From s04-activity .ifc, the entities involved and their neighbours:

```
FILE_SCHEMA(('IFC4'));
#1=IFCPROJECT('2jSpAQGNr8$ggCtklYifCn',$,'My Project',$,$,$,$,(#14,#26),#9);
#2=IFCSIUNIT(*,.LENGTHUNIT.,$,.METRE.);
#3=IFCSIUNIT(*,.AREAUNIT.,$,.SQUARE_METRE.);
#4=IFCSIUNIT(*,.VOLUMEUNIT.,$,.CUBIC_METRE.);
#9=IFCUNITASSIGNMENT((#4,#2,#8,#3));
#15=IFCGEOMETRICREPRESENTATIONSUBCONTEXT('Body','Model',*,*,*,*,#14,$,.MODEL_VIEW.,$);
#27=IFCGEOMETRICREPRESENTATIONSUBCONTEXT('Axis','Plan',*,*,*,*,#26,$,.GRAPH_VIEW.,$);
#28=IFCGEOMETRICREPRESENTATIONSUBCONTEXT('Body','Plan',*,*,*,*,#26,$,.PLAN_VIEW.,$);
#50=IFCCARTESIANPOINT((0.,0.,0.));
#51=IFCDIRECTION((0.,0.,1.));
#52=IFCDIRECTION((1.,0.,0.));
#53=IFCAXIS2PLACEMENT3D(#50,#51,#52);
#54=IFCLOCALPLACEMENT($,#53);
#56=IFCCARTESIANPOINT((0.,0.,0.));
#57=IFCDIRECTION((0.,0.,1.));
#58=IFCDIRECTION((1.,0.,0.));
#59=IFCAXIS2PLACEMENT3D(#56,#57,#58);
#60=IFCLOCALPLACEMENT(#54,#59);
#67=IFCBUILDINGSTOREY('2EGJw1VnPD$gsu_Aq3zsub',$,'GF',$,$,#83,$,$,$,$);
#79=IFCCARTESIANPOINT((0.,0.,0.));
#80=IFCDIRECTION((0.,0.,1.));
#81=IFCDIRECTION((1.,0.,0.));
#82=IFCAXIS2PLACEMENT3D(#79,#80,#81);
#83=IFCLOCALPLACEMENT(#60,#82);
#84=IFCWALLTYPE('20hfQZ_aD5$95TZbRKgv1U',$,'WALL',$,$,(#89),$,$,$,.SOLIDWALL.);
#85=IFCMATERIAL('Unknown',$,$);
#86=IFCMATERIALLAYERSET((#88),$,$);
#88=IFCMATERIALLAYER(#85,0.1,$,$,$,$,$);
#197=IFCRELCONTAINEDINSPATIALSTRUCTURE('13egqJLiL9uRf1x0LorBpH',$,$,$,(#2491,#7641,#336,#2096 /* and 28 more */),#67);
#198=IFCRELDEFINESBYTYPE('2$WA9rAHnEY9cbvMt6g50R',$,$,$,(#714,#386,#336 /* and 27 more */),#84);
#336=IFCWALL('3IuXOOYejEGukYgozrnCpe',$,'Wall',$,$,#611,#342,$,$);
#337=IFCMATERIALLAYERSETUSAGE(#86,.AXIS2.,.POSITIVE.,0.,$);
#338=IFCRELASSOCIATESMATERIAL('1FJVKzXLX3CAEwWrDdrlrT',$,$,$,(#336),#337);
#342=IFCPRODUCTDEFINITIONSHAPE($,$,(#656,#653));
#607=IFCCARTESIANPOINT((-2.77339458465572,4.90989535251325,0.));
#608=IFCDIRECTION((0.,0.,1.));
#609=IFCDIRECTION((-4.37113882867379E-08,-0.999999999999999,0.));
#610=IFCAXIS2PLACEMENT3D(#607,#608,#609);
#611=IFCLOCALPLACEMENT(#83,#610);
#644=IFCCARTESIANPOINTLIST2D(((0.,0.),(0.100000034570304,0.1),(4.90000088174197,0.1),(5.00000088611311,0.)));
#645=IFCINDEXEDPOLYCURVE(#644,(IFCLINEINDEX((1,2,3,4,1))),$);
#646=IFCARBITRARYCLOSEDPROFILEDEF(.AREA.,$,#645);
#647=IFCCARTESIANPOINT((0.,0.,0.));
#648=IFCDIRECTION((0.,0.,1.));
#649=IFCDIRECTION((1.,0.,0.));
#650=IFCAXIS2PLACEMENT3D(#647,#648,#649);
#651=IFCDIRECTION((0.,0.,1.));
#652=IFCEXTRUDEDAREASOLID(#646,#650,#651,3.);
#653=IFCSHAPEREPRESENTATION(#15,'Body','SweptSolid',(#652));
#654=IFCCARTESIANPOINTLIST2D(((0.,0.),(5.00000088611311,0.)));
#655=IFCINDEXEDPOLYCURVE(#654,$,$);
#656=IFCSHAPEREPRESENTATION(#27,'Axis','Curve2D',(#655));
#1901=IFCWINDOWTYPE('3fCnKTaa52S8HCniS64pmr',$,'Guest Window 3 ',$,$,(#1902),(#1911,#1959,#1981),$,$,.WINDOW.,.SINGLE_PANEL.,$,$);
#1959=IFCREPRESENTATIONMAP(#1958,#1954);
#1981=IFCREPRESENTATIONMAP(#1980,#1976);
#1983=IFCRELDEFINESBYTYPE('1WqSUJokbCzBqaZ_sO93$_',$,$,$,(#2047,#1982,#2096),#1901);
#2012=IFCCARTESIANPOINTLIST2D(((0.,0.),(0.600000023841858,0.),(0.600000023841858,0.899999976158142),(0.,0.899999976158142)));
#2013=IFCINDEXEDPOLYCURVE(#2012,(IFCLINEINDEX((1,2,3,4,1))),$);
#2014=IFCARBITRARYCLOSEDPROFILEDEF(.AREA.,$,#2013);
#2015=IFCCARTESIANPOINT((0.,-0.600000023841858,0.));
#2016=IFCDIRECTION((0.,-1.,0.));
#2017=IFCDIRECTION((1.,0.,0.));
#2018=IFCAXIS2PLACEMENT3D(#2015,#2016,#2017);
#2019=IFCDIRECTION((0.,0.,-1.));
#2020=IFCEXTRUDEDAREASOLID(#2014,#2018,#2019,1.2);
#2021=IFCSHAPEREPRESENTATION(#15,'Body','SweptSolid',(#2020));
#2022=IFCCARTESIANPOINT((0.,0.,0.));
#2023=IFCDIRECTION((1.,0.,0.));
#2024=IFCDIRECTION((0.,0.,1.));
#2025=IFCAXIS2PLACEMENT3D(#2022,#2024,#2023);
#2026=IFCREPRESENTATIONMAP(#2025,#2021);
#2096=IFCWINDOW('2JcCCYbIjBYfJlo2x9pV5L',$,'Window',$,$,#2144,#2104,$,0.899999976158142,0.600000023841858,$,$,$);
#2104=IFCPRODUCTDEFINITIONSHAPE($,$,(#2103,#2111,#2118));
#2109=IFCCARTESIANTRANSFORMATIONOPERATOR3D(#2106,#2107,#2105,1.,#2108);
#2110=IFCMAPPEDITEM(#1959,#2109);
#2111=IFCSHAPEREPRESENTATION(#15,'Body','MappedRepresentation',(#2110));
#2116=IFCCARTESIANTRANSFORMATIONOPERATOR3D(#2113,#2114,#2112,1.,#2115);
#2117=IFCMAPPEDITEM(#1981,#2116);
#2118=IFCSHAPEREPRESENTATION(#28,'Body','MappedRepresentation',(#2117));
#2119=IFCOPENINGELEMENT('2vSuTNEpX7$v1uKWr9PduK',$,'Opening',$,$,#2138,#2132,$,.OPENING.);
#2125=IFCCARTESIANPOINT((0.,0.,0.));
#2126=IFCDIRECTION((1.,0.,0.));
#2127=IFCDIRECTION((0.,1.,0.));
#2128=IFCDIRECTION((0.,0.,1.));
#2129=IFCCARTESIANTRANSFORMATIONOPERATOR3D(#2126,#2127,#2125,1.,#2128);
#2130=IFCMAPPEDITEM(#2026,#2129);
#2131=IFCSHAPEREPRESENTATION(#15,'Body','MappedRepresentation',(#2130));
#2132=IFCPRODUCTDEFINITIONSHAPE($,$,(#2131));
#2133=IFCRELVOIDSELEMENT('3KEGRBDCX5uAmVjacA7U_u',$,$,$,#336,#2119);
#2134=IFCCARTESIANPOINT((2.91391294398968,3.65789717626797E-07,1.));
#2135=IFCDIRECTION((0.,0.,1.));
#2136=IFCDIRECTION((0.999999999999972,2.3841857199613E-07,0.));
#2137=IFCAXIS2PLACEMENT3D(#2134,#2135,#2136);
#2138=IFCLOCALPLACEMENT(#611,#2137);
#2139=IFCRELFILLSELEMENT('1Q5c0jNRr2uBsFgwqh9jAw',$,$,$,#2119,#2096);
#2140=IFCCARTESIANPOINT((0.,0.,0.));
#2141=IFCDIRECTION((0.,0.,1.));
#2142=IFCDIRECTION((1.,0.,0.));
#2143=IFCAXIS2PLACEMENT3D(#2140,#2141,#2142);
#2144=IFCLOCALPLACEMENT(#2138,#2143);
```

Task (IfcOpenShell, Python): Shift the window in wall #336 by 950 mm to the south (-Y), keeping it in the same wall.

```python
import ifcopenshell
import ifcopenshell.api.geometry
import ifcopenshell.util.placement
import ifcopenshell.util.unit

model = ifcopenshell.open("s04-activity .ifc")
unit_scale = ifcopenshell.util.unit.calculate_unit_scale(model)

window = model.by_id(2096)
opening = window.FillsVoids[0].RelatingOpeningElement
wall = opening.VoidsElements[0].RelatingBuildingElement

wall_matrix = ifcopenshell.util.placement.get_local_placement(wall.ObjectPlacement)
shift = wall_matrix[:3, 0] * 0.95 / unit_scale
before = ifcopenshell.util.placement.get_local_placement(window.ObjectPlacement)[:3, 3].copy()

# The window is placed relative to its opening, so it follows when the opening moves.
matrix = ifcopenshell.util.placement.get_local_placement(opening.ObjectPlacement)
matrix[:3, 3] += shift
ifcopenshell.api.geometry.edit_object_placement(
    model, product=opening, matrix=matrix, is_si=False, should_transform_children=True
)

after = ifcopenshell.util.placement.get_local_placement(window.ObjectPlacement)[:3, 3]
print("window moved by", (after - before).round(3) + 0.0)

model.write("s04-activity _rev.ifc")
```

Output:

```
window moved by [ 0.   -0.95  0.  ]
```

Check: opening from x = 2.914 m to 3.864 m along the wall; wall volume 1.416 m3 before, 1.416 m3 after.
